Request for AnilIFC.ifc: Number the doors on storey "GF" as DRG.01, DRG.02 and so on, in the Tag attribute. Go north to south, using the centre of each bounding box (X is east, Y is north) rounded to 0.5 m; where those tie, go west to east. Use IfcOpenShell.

First a look at what the model holds.

```python
import ifcopenshell
import ifcopenshell.util.element
import ifcopenshell.util.placement

model = ifcopenshell.open("AnilIFC.ifc")
print(model.schema)
storey = next(s for s in model.by_type("IfcBuildingStorey") if s.Name == "GF")
doors = [e for e in ifcopenshell.util.element.get_decomposition(storey) if e.is_a("IfcDoor")]
for e in sorted(doors, key=lambda e: e.id()):
    origin = ifcopenshell.util.placement.get_local_placement(e.ObjectPlacement)[:3, 3]
    print(e.id(), e.Tag, e.Name, origin.round(2) + 0.0, sep=" | ")
```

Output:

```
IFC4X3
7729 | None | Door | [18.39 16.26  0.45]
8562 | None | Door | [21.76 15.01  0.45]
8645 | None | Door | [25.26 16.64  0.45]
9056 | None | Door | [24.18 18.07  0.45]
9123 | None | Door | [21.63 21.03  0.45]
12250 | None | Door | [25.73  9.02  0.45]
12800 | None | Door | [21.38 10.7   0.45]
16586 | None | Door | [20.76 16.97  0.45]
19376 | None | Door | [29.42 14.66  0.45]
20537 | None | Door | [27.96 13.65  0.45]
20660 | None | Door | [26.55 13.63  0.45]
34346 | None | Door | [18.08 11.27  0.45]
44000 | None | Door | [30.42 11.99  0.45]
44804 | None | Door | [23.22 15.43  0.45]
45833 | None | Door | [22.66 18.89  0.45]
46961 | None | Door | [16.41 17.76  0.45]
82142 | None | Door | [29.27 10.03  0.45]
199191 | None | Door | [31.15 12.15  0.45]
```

```python
import ifcopenshell
import ifcopenshell.geom
import ifcopenshell.util.element
import ifcopenshell.util.shape

model = ifcopenshell.open("AnilIFC.ifc")
settings = ifcopenshell.geom.settings()
settings.set("use-world-coords", True)


def centre(element):
    shape = ifcopenshell.geom.create_shape(settings, element)
    return ifcopenshell.util.shape.get_bbox_centroid(shape.geometry)


storey = next(s for s in model.by_type("IfcBuildingStorey") if s.Name == "GF")
doors = [e for e in ifcopenshell.util.element.get_decomposition(storey) if e.is_a("IfcDoor")]

# Insertion points can sit at a corner or the storey origin, so sort by the geometry (in metres).
centres = {e: centre(e) for e in doors}
doors.sort(key=lambda e: (-round(centres[e][1] / 0.5), centres[e][0]))

for i, e in enumerate(doors, start=1):
    number = f"DRG.{i:02d}"
    e.Tag = number
    print(e.id(), number)

model.write("AnilIFC_rev.ifc")
```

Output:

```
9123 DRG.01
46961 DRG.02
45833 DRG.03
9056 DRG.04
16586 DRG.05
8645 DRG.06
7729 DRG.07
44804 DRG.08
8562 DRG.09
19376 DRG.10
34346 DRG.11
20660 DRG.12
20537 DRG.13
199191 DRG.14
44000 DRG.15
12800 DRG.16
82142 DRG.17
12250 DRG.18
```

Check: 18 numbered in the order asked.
